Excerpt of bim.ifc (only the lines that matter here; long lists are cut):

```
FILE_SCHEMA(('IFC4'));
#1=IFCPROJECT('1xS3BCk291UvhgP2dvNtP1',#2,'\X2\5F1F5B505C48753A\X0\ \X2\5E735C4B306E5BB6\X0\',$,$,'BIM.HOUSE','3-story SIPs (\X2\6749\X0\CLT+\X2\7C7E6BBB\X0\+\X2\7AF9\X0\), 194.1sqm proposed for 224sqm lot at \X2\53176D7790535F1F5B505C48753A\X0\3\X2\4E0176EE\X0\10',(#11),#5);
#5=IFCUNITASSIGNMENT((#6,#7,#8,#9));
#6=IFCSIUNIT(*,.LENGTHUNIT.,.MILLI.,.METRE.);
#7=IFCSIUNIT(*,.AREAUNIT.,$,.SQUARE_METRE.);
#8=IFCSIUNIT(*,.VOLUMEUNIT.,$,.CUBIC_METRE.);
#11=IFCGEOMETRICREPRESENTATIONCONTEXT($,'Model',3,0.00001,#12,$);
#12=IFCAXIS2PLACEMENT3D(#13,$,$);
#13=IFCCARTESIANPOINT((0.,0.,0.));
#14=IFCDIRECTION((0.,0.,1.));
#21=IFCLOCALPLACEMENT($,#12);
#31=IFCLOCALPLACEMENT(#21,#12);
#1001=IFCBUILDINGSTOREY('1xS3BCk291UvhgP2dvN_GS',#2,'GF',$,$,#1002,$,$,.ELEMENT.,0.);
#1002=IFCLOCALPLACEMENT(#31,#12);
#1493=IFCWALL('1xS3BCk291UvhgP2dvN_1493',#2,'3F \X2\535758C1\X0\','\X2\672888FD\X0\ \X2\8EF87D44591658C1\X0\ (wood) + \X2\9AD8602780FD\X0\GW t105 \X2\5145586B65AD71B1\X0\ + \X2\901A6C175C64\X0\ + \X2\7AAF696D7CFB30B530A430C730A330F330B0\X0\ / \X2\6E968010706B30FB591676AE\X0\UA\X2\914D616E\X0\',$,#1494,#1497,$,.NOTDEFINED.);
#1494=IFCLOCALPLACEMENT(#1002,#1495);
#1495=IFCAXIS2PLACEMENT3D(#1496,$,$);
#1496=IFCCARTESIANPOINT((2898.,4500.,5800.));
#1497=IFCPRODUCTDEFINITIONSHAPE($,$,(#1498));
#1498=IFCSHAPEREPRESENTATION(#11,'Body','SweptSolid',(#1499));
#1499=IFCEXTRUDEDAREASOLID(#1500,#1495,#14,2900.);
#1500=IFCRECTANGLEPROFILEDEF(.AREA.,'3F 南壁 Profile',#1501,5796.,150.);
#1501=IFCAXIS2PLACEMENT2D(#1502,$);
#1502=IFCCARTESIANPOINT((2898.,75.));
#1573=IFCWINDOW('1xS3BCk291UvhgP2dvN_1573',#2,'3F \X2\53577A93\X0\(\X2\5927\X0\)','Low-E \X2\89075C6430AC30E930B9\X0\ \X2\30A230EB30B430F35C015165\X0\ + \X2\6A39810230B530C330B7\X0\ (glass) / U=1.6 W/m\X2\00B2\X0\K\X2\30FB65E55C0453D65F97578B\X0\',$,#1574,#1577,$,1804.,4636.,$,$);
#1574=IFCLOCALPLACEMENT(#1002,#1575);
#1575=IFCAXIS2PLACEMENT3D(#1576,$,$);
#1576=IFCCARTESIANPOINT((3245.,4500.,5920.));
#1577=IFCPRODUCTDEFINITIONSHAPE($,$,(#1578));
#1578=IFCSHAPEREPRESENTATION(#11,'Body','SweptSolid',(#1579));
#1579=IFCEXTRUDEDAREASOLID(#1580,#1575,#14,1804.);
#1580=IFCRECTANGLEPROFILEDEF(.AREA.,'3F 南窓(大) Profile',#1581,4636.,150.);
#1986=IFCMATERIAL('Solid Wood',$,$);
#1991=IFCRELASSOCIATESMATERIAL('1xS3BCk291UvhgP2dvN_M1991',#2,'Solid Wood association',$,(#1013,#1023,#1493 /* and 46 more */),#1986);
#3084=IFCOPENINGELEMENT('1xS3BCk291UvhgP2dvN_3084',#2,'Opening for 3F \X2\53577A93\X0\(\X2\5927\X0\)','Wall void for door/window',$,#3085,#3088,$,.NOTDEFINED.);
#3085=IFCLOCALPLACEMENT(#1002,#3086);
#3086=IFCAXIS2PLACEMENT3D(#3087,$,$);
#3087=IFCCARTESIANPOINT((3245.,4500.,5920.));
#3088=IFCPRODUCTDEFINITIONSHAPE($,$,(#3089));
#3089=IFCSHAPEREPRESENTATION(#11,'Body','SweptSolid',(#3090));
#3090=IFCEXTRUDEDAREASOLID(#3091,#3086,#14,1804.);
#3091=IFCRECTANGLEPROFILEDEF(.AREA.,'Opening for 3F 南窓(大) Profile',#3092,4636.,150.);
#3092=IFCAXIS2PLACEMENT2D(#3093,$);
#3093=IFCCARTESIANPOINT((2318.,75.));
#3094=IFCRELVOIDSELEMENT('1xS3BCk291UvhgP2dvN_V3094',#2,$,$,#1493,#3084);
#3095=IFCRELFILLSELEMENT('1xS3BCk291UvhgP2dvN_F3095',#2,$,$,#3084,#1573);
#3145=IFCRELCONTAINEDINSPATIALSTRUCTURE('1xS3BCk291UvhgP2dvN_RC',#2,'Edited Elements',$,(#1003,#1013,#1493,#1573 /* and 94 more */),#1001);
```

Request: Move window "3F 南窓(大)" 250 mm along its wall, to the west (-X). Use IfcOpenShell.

```python
import ifcopenshell
import ifcopenshell.api.geometry
import ifcopenshell.util.placement
import ifcopenshell.util.unit

model = ifcopenshell.open("bim.ifc")
unit_scale = ifcopenshell.util.unit.calculate_unit_scale(model)

window = model.by_guid("1xS3BCk291UvhgP2dvN_1573")
opening = window.FillsVoids[0].RelatingOpeningElement
wall = opening.VoidsElements[0].RelatingBuildingElement

wall_matrix = ifcopenshell.util.placement.get_local_placement(wall.ObjectPlacement)
shift = wall_matrix[:3, 0] * -0.25 / unit_scale
before = ifcopenshell.util.placement.get_local_placement(window.ObjectPlacement)[:3, 3].copy()

# The window is not placed relative to its opening, so move both.
for product in (opening, window):
    matrix = ifcopenshell.util.placement.get_local_placement(product.ObjectPlacement)
    matrix[:3, 3] += shift
    ifcopenshell.api.geometry.edit_object_placement(model, product=product, matrix=matrix, is_si=False)

after = ifcopenshell.util.placement.get_local_placement(window.ObjectPlacement)[:3, 3]
print("window moved by", (after - before).round(3) + 0.0)

model.write("bim_v2.ifc")
```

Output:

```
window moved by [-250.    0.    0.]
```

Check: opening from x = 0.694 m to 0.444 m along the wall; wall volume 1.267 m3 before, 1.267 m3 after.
